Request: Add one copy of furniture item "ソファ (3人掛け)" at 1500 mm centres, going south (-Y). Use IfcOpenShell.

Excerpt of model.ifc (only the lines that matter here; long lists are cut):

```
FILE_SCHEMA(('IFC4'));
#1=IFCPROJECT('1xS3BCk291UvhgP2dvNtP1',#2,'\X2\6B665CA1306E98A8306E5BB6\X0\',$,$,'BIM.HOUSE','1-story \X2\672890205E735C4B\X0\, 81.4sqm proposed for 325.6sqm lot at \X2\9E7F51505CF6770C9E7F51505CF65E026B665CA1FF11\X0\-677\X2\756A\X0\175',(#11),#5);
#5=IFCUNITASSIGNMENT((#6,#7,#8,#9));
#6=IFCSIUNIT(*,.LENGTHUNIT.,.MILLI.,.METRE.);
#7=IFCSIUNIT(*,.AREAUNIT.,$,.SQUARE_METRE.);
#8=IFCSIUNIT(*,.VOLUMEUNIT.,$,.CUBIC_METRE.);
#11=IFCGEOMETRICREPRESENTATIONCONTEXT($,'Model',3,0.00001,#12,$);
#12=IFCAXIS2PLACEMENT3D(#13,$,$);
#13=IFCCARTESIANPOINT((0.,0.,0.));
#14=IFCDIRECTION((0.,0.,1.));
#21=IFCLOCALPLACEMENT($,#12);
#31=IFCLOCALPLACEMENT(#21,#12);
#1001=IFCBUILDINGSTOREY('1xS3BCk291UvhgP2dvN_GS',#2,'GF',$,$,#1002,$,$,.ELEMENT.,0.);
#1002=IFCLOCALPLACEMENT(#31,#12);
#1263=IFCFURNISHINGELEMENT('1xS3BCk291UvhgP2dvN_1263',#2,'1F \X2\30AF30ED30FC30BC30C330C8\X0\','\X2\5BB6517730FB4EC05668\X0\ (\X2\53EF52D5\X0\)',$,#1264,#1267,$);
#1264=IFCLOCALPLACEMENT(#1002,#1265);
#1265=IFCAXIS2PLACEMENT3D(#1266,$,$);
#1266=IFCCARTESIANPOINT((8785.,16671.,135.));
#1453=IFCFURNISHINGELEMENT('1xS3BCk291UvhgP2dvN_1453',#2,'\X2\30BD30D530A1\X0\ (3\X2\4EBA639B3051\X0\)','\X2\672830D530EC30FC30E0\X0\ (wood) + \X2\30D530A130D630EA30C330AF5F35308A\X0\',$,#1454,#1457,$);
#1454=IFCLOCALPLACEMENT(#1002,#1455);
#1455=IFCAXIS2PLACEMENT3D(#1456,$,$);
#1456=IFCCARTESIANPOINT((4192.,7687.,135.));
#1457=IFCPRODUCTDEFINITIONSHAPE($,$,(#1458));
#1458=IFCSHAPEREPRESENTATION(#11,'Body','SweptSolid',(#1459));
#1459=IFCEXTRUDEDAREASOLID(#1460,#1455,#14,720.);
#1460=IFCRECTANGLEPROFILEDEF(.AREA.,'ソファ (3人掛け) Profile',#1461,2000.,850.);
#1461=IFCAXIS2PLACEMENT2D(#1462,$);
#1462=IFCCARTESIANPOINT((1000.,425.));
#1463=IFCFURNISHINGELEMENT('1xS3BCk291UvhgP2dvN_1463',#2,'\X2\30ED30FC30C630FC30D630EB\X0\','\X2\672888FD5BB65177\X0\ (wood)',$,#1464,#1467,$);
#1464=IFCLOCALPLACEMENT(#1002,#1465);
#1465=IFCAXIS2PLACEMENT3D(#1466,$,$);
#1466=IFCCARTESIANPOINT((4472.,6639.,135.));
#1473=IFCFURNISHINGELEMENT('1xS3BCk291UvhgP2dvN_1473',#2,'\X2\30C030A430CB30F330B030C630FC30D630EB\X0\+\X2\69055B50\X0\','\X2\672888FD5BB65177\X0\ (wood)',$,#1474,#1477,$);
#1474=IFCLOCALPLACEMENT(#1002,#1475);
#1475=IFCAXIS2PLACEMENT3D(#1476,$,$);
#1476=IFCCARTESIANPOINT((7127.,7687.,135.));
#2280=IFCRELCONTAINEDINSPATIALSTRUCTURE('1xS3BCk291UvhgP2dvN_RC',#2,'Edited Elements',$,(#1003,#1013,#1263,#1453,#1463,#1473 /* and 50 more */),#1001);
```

```python
import numpy as np
import ifcopenshell
import ifcopenshell.api.geometry
import ifcopenshell.api.root
import ifcopenshell.util.element
import ifcopenshell.util.placement

model = ifcopenshell.open("model.ifc")


def reuse_history(source, copy):
    """copy_class also copies each property set's owner history, people and application; keep the originals."""
    for rel in copy.IsDefinedBy:
        if rel.is_a("IfcRelDefinesByProperties") and (history := rel.RelatingPropertyDefinition.OwnerHistory):
            rel.RelatingPropertyDefinition.OwnerHistory = source.OwnerHistory
            ifcopenshell.util.element.remove_deep2(model, history)


source = model.by_guid("1xS3BCk291UvhgP2dvN_1453")
base = ifcopenshell.util.placement.get_local_placement(source.ObjectPlacement)
step = np.array([0.0, -1.0, 0.0]) * 1500.0

for i in range(1, 2):
    copy = ifcopenshell.api.root.copy_class(model, product=source)
    copy.Representation = ifcopenshell.util.element.copy_deep(
        model, source.Representation, exclude=["IfcGeometricRepresentationContext", "IfcRepresentationMap"]
    )
    reuse_history(source, copy)
    matrix = base.copy()
    matrix[:3, 3] += i * step
    print("added at", matrix[:3, 3].round(3) + 0.0)
    ifcopenshell.api.geometry.edit_object_placement(model, product=copy, matrix=matrix, is_si=False)

model.write("model_edited.ifc")
```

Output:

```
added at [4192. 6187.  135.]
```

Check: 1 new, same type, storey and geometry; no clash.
